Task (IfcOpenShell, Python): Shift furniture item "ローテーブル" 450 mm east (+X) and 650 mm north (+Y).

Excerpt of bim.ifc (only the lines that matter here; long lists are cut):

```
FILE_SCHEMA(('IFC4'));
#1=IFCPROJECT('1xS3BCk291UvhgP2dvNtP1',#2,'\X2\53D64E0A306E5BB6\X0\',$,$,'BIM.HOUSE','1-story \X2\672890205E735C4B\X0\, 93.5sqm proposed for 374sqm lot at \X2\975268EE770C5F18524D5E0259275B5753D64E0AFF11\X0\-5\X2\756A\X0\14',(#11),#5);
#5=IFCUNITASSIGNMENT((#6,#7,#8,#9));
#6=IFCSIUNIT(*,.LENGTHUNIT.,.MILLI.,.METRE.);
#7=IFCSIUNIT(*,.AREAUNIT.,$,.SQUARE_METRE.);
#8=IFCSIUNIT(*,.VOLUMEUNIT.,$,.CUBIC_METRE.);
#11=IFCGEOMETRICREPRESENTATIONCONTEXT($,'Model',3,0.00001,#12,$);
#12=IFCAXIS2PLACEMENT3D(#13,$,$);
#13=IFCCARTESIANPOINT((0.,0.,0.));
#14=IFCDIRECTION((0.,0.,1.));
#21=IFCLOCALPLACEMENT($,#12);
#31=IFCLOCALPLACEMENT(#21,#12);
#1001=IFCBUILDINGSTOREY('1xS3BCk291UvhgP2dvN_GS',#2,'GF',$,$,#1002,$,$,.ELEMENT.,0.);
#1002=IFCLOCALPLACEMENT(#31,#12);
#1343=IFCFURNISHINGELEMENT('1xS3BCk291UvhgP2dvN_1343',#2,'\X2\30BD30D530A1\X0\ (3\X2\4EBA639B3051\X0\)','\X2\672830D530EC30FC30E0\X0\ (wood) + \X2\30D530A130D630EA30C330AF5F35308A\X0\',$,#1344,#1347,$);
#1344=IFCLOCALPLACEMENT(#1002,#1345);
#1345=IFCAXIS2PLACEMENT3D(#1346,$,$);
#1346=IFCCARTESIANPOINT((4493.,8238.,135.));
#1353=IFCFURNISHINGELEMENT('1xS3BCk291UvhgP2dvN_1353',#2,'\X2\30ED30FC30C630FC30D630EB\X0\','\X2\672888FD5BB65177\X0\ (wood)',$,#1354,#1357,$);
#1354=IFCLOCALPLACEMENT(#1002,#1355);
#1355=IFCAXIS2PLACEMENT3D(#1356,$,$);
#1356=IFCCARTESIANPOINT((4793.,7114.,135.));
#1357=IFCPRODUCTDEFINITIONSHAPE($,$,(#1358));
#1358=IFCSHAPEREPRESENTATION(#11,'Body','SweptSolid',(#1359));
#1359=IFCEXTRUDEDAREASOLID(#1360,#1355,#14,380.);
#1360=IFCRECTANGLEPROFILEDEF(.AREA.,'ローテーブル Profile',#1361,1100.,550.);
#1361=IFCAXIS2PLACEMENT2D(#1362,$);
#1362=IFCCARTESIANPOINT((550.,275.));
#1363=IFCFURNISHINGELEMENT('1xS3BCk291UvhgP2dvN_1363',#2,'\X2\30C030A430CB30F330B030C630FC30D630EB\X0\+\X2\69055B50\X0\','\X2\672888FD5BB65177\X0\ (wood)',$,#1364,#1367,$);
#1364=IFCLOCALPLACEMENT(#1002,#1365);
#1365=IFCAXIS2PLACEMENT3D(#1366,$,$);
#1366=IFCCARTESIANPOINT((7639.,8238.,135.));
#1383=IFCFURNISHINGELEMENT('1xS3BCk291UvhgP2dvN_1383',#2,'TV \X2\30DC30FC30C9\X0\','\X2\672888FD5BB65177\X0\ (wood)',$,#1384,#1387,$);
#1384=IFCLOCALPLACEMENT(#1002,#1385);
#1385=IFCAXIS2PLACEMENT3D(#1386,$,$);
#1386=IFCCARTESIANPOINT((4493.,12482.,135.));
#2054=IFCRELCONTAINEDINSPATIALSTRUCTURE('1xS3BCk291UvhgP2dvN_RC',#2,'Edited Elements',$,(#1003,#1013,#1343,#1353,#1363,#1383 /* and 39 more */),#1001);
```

```python
import ifcopenshell
import ifcopenshell.api.geometry
import ifcopenshell.util.placement

model = ifcopenshell.open("bim.ifc")

item = model.by_guid("1xS3BCk291UvhgP2dvN_1353")
matrix = ifcopenshell.util.placement.get_local_placement(item.ObjectPlacement)
matrix[0, 3] += 450.0
matrix[1, 3] += 650.0
ifcopenshell.api.geometry.edit_object_placement(model, product=item, matrix=matrix, is_si=False)

print(ifcopenshell.util.placement.get_local_placement(item.ObjectPlacement).round(3) + 0.0)

model.write("bim_v2.ifc")
```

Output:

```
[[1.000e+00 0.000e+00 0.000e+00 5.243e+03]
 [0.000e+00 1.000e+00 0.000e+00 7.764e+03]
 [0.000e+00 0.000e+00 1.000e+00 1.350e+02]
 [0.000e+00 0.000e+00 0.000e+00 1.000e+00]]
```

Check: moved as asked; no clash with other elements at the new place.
